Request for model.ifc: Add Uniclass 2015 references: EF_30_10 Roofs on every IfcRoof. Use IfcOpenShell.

First a look at what the model holds.

```python
import ifcopenshell

model = ifcopenshell.open("model.ifc")
print(model.schema)
print("classifications:", [c.Name for c in model.by_type("IfcClassification")])
for ifc_class in ("IfcDoor", "IfcRoof", "IfcStair", "IfcWall", "IfcWindow"):
    print(ifc_class, len(model.by_type(ifc_class)))
```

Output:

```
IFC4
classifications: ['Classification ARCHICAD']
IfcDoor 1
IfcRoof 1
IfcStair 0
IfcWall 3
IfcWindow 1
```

```python
import ifcopenshell
import ifcopenshell.api.classification

model = ifcopenshell.open("model.ifc")

system = ifcopenshell.api.classification.add_classification(model, classification="Uniclass 2015")

codes = {
    "IfcRoof": ("EF_30_10", "Roofs"),
}
for ifc_class, (code, name) in codes.items():
    products = model.by_type(ifc_class)
    ifcopenshell.api.classification.add_reference(
        model, products=products, classification=system, identification=code, name=name
    )
    print(code, len(products))

model.write("model-out.ifc")
```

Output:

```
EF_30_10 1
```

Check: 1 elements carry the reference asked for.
